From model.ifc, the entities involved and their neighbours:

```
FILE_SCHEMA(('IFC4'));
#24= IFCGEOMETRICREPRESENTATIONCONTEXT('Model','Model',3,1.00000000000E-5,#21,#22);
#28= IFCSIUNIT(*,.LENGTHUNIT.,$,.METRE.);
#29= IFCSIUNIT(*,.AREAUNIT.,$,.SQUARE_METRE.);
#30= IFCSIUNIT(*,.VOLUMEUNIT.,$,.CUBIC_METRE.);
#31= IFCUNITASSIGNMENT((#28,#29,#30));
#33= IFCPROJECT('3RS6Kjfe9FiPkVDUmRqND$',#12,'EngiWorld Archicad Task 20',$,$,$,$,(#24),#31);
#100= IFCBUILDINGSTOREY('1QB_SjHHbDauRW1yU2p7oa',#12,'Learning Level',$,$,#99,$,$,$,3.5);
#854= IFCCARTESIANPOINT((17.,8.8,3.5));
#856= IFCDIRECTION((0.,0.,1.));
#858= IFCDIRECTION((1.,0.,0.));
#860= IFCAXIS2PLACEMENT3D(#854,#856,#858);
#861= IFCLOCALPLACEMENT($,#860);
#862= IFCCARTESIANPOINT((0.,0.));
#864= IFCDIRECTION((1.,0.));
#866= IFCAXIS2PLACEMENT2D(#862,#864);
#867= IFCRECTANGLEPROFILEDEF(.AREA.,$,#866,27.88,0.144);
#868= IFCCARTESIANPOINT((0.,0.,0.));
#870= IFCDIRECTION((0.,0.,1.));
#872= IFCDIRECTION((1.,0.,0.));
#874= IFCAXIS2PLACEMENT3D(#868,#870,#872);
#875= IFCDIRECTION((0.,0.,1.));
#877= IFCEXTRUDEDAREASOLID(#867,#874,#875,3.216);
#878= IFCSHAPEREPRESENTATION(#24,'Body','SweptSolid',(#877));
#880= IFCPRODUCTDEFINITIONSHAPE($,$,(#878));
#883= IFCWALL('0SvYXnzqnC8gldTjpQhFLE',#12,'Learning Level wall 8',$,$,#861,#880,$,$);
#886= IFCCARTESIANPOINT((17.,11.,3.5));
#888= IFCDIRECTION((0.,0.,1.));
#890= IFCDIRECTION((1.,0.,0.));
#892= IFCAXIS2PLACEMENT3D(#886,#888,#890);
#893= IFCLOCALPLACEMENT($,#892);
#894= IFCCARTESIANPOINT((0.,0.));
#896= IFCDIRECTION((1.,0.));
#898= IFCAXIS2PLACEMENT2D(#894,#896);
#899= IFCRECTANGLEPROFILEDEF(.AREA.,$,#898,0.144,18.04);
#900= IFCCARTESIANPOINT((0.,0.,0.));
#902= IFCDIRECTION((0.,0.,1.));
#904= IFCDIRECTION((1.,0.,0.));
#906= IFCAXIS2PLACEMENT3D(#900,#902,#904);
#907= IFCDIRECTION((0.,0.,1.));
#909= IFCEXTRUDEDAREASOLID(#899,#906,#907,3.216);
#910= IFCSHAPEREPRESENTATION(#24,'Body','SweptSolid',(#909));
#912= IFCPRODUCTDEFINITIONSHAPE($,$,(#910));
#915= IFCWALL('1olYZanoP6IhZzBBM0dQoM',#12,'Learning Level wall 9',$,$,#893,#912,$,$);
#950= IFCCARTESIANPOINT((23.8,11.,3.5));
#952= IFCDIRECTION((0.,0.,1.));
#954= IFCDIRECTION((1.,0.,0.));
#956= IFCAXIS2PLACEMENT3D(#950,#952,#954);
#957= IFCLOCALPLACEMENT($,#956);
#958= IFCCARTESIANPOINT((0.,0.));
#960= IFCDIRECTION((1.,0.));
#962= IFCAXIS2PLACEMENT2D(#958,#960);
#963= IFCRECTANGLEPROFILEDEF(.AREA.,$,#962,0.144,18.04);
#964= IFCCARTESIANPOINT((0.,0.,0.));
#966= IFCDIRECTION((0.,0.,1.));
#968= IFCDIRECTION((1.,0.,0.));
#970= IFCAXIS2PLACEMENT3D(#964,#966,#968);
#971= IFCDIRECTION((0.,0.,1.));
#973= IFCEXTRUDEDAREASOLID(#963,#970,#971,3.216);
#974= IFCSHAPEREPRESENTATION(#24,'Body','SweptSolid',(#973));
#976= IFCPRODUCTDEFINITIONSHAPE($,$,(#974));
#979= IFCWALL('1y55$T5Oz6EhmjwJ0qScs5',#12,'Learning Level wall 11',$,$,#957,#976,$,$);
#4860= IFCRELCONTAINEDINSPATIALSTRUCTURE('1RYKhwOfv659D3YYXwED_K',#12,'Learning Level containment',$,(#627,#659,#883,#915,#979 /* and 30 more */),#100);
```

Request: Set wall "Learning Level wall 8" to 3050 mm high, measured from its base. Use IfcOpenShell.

```python
import ifcopenshell
import ifcopenshell.geom
import ifcopenshell.util.shape

model = ifcopenshell.open("model.ifc")
settings = ifcopenshell.geom.settings()


def volume(element):
    """Net volume in cubic metres, openings subtracted."""
    shape = ifcopenshell.geom.create_shape(settings, element)
    return ifcopenshell.util.shape.get_volume(shape.geometry)


wall = model.by_guid("0SvYXnzqnC8gldTjpQhFLE")
before = volume(wall)

body = next(r for r in wall.Representation.Representations if r.RepresentationIdentifier == "Body")
solid = body.Items[0]
old_height = solid.Depth
solid.Depth = 3.05
after = volume(wall)

print(f"height {old_height:g} -> {solid.Depth:g}, volume {before:.3f} -> {after:.3f} m3")

model.write("model_v2.ifc")
```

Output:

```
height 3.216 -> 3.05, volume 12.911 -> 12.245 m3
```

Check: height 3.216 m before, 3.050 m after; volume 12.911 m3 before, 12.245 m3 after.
